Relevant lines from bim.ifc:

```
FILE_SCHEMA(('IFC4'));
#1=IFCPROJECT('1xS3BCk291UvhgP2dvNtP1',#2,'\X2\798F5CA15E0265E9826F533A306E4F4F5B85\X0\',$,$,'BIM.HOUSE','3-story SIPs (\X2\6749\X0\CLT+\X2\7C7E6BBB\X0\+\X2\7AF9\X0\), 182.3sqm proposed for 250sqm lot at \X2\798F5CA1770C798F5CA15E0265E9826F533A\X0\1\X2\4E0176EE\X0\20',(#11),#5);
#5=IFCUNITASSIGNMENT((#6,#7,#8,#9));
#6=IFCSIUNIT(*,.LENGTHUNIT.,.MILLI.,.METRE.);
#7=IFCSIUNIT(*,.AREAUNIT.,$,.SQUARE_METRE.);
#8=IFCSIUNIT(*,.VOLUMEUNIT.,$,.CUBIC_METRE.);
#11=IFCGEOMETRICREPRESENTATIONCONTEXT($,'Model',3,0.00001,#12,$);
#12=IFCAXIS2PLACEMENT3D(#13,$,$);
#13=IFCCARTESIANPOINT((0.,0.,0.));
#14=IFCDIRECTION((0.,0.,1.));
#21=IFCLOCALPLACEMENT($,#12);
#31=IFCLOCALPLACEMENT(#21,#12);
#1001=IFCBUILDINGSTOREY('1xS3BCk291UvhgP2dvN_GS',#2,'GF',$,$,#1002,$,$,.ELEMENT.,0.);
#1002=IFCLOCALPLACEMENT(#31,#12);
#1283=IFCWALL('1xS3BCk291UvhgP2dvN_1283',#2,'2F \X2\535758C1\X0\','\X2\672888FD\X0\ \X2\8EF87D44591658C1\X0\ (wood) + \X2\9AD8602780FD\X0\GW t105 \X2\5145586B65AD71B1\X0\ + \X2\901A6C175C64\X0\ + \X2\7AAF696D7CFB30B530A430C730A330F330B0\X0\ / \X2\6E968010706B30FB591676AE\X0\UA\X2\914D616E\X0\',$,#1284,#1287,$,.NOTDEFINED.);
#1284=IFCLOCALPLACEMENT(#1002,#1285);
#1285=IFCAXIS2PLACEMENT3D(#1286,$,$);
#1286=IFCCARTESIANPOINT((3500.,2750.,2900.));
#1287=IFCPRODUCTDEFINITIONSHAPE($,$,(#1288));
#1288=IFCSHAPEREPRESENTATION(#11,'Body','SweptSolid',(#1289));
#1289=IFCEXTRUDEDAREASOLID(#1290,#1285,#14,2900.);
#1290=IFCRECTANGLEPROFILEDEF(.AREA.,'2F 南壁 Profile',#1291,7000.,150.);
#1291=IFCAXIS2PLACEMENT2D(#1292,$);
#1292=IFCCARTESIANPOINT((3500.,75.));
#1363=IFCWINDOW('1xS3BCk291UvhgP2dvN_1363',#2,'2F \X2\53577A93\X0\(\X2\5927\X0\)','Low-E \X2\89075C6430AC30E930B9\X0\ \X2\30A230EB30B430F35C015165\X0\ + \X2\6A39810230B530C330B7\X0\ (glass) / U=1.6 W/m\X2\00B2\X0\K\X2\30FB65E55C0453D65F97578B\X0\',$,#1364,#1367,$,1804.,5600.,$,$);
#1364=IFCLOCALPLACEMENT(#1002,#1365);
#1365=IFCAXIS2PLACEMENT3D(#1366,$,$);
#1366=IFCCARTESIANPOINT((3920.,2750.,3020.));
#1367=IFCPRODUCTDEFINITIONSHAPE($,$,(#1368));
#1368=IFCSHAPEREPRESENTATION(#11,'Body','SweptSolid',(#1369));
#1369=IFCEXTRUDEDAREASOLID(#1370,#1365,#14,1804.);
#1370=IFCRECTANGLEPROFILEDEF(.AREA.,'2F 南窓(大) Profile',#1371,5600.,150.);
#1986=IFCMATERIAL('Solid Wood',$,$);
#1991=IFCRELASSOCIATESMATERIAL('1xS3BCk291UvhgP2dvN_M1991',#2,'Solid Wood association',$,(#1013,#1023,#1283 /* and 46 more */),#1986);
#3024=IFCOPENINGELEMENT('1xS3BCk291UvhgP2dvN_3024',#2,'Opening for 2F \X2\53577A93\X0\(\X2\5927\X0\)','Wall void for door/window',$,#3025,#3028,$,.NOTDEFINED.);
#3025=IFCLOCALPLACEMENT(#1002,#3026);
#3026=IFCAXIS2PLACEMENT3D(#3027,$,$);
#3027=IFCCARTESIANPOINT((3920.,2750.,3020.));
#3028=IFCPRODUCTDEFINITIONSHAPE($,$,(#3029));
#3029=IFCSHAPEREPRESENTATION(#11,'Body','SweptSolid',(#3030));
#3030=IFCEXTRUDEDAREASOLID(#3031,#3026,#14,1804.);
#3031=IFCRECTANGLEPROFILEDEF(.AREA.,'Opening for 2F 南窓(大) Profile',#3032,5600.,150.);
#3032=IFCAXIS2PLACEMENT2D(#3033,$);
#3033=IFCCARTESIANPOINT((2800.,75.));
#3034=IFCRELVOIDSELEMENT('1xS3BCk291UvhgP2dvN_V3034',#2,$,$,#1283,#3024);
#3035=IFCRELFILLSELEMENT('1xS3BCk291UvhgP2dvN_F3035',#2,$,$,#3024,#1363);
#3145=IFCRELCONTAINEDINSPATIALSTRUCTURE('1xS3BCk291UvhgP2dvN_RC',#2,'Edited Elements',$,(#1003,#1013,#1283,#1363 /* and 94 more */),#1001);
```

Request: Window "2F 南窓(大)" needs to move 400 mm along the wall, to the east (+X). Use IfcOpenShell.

```python
import ifcopenshell
import ifcopenshell.api.geometry
import ifcopenshell.util.placement
import ifcopenshell.util.unit

model = ifcopenshell.open("bim.ifc")
unit_scale = ifcopenshell.util.unit.calculate_unit_scale(model)

window = model.by_guid("1xS3BCk291UvhgP2dvN_1363")
opening = window.FillsVoids[0].RelatingOpeningElement
wall = opening.VoidsElements[0].RelatingBuildingElement

wall_matrix = ifcopenshell.util.placement.get_local_placement(wall.ObjectPlacement)
shift = wall_matrix[:3, 0] * 0.4 / unit_scale
before = ifcopenshell.util.placement.get_local_placement(window.ObjectPlacement)[:3, 3].copy()

# The window is not placed relative to its opening, so move both.
for product in (opening, window):
    matrix = ifcopenshell.util.placement.get_local_placement(product.ObjectPlacement)
    matrix[:3, 3] += shift
    ifcopenshell.api.geometry.edit_object_placement(model, product=product, matrix=matrix, is_si=False)

after = ifcopenshell.util.placement.get_local_placement(window.ObjectPlacement)[:3, 3]
print("window moved by", (after - before).round(3) + 0.0)

model.write("bim_rev.ifc")
```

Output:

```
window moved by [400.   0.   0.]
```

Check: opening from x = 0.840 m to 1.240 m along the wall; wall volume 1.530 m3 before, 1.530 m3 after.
